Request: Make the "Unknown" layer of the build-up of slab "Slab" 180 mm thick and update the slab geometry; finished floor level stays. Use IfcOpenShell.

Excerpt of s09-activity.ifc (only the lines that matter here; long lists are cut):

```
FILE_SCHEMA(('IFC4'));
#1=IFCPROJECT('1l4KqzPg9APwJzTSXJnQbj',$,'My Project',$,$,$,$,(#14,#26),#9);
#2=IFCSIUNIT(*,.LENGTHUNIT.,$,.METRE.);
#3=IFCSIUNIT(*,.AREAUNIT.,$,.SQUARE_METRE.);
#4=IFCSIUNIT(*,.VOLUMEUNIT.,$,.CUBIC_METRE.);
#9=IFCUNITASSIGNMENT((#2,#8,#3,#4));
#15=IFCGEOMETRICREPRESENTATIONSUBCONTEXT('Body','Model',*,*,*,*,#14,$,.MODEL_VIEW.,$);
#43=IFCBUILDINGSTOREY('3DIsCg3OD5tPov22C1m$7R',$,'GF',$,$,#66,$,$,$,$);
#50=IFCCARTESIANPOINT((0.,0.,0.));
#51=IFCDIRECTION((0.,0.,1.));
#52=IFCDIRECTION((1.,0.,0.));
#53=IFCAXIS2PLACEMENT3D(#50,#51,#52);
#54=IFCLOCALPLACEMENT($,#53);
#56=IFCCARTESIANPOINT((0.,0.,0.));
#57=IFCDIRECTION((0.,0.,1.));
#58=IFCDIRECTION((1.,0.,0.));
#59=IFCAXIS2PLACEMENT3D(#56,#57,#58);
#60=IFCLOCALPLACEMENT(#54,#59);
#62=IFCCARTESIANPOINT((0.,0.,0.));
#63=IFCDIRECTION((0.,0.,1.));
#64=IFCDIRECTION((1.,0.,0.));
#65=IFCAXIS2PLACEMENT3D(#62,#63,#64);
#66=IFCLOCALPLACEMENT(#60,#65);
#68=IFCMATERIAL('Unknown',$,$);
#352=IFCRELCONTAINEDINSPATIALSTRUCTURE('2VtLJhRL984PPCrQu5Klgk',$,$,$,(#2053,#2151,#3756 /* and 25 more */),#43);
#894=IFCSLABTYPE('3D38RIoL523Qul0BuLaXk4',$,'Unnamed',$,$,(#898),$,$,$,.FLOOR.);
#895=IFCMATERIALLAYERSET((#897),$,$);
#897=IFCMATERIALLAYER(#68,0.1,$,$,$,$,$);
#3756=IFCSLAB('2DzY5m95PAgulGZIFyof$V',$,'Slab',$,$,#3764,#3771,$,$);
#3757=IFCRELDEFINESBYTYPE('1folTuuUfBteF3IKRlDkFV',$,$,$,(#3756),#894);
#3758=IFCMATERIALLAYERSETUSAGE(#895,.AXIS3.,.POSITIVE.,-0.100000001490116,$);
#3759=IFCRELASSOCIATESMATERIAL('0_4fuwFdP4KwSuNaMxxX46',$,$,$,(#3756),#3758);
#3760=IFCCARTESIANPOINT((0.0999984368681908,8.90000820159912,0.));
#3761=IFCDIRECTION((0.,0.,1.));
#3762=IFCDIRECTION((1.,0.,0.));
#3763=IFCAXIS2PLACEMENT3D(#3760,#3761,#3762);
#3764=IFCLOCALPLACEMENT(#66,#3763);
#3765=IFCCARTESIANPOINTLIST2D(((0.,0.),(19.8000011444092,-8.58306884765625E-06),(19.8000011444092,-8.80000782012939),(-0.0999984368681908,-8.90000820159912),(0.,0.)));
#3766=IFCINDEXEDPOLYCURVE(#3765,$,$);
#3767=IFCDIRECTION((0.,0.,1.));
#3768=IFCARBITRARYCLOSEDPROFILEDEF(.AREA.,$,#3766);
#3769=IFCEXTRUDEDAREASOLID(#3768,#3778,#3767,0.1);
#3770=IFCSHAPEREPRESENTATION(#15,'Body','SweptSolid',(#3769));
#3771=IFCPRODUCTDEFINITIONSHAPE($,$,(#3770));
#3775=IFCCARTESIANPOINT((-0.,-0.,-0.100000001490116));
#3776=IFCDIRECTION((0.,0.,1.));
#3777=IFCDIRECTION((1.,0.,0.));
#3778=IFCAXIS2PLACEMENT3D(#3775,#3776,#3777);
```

```python
import ifcopenshell
import ifcopenshell.util.element
import ifcopenshell.util.representation

model = ifcopenshell.open("s09-activity.ifc")

layer_set = model.by_id(895)
layer = next(l for l in layer_set.MaterialLayers if l.Material and l.Material.Name == "Unknown")
change = 0.18 - layer.LayerThickness
layer.LayerThickness += change

# Geometry does not follow the layer set by itself.
slabs = [e for e in ifcopenshell.util.element.get_elements_by_material(model, layer_set) if e.is_a("IfcSlab")]
for slab in sorted(slabs, key=lambda e: e.id()):
    body = ifcopenshell.util.representation.get_representation(slab, "Model", "Body")
    solid = body.Items[0]
    old_depth = solid.Depth
    solid.Depth += change
    # Extruded upwards: lower the start of the extrusion so the top stays.
    x, y, z = solid.Position.Location.Coordinates
    solid.Position.Location = model.createIfcCartesianPoint((x, y, z - change))
    print(slab.id(), f"{old_depth:g} -> {solid.Depth:g}")

# The layers are counted up from the underside, which has moved.
for usage in {ifcopenshell.util.element.get_material(slab) for slab in slabs}:
    usage.OffsetFromReferenceLine -= change

model.write("s09-activity_v2.ifc")
```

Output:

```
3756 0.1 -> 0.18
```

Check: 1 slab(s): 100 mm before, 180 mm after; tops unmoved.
